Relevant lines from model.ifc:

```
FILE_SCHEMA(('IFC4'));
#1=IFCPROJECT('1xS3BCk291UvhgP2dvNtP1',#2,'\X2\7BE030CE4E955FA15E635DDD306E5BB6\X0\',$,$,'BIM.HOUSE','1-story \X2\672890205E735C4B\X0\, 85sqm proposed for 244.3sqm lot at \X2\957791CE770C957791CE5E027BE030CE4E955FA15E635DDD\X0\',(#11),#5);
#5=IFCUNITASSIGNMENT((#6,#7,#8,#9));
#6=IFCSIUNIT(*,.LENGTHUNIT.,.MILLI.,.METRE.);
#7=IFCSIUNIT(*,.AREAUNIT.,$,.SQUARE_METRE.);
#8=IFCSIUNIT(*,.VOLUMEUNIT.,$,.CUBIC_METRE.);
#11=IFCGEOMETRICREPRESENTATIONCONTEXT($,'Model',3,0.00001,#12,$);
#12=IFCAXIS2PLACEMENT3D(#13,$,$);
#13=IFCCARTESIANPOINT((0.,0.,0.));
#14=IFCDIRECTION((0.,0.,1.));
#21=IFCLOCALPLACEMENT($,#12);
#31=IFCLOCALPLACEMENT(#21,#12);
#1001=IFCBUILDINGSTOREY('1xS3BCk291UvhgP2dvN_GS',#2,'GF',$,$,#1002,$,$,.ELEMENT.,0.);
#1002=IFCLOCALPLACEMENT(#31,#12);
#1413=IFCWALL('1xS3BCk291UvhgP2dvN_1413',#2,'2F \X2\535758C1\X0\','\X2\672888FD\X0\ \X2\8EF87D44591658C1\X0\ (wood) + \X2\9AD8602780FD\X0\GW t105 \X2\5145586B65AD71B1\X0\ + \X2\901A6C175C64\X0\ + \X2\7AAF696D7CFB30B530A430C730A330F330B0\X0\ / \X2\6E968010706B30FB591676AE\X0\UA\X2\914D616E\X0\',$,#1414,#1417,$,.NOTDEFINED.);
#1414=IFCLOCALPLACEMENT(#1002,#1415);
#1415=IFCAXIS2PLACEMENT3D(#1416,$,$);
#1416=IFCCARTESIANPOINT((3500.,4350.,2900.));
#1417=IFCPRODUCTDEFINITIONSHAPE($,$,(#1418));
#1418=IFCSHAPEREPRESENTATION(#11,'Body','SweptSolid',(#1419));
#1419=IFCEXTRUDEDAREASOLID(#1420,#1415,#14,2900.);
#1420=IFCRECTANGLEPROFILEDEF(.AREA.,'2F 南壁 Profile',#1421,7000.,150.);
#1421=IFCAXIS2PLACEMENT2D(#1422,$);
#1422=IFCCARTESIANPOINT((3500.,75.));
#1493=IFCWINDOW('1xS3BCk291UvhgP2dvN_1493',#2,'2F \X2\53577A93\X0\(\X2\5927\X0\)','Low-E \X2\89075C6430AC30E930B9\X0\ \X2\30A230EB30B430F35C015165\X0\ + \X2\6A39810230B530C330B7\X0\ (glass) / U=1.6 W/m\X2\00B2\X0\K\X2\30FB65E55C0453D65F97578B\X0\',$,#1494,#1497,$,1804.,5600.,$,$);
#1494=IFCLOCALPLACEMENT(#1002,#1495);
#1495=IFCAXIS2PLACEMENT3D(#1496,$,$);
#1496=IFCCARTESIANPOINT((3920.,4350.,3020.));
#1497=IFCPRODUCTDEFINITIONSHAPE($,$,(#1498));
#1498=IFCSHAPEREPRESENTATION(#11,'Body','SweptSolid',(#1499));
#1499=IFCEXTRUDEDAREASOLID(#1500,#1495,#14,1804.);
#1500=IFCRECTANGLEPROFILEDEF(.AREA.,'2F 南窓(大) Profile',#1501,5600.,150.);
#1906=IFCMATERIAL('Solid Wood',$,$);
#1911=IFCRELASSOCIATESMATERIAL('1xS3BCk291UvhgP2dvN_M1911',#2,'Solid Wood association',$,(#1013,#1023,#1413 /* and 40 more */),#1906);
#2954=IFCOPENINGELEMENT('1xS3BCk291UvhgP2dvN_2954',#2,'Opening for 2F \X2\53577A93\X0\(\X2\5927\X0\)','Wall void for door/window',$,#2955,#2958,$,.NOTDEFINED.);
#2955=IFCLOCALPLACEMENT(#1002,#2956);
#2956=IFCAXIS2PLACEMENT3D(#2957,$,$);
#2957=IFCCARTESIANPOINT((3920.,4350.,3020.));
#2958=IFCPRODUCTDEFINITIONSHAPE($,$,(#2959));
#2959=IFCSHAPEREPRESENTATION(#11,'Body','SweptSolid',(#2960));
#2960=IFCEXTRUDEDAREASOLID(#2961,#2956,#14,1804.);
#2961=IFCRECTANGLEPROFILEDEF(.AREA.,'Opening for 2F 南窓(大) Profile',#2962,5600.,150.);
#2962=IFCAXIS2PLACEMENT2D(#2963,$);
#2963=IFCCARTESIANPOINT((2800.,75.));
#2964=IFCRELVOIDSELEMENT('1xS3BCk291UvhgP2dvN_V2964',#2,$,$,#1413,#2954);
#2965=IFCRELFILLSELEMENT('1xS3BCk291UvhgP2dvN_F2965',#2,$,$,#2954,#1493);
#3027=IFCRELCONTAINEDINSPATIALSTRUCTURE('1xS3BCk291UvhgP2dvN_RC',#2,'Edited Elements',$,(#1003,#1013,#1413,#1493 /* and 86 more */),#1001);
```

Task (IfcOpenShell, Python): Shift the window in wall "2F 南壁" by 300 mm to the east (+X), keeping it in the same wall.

```python
import ifcopenshell
import ifcopenshell.api.geometry
import ifcopenshell.util.placement

model = ifcopenshell.open("model.ifc")

window = model.by_id(1493)
opening = window.FillsVoids[0].RelatingOpeningElement
wall = opening.VoidsElements[0].RelatingBuildingElement

wall_matrix = ifcopenshell.util.placement.get_local_placement(wall.ObjectPlacement)
shift = wall_matrix[:3, 0] * 300.0
before = ifcopenshell.util.placement.get_local_placement(window.ObjectPlacement)[:3, 3].copy()

# The window is not placed relative to its opening, so move both.
for product in (opening, window):
    matrix = ifcopenshell.util.placement.get_local_placement(product.ObjectPlacement)
    matrix[:3, 3] += shift
    ifcopenshell.api.geometry.edit_object_placement(model, product=product, matrix=matrix, is_si=False)

after = ifcopenshell.util.placement.get_local_placement(window.ObjectPlacement)[:3, 3]
print("window moved by", (after - before).round(3) + 0.0)

model.write("model-out.ifc")
```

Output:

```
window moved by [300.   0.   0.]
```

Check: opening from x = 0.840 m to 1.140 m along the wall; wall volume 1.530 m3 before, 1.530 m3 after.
